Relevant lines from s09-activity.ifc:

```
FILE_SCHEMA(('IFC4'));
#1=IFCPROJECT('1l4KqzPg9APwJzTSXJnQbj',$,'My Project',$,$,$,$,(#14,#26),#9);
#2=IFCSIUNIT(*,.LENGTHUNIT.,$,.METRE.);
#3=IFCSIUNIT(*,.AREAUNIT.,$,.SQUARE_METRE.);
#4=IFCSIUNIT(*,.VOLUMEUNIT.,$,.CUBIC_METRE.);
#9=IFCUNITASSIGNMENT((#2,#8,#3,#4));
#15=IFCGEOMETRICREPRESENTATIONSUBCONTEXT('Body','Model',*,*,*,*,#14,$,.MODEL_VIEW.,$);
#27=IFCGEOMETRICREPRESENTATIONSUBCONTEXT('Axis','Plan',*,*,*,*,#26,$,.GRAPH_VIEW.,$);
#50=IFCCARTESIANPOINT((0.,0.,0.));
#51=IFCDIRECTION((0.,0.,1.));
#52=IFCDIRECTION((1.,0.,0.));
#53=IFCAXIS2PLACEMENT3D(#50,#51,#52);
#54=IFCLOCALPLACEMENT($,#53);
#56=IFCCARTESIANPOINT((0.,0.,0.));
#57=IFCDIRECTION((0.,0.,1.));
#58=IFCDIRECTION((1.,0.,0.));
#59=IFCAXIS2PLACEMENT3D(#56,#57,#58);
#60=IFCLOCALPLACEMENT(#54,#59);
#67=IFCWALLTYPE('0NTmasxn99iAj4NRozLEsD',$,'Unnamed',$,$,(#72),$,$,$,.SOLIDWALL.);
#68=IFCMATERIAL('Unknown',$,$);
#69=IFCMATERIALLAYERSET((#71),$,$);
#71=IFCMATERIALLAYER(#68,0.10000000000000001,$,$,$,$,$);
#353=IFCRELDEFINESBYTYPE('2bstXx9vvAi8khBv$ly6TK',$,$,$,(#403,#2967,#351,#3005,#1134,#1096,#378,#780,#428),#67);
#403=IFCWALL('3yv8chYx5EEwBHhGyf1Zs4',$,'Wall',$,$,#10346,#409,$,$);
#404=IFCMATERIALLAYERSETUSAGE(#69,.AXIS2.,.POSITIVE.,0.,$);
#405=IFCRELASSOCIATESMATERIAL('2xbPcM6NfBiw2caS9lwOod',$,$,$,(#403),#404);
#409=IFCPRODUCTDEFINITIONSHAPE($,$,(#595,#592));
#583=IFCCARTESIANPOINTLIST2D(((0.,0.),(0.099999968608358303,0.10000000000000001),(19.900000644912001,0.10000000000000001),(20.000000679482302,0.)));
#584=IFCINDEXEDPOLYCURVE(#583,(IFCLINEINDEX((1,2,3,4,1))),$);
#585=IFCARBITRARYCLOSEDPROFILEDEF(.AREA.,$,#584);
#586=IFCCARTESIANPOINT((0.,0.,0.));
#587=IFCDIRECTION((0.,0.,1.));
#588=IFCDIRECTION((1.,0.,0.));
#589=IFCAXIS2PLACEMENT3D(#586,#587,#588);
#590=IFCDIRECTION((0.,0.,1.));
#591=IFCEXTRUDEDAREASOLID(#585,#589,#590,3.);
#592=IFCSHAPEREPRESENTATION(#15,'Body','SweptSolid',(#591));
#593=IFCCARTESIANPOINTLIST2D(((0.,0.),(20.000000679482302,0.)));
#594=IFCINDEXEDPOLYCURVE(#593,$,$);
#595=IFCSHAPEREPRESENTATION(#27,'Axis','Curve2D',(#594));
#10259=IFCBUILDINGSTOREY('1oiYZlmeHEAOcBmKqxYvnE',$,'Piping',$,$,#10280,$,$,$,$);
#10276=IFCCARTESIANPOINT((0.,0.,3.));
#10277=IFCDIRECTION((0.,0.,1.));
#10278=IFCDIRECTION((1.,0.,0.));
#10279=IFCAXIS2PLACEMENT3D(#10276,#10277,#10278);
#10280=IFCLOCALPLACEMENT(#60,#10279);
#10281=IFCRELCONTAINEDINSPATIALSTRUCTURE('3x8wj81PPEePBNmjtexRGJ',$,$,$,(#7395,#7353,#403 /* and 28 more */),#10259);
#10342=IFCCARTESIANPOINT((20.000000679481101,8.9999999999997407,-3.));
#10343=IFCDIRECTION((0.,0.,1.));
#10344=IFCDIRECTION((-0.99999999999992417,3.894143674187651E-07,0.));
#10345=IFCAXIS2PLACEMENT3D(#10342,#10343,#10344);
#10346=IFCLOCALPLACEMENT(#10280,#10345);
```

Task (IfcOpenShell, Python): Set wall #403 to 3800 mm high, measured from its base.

```python
import ifcopenshell
import ifcopenshell.geom
import ifcopenshell.util.representation
import ifcopenshell.util.shape
import ifcopenshell.util.unit

model = ifcopenshell.open("s09-activity.ifc")
unit_scale = ifcopenshell.util.unit.calculate_unit_scale(model)
settings = ifcopenshell.geom.settings()


def volume(element):
    """Net volume in cubic metres, openings subtracted."""
    shape = ifcopenshell.geom.create_shape(settings, element)
    return ifcopenshell.util.shape.get_volume(shape.geometry)


wall = model.by_guid("3yv8chYx5EEwBHhGyf1Zs4")
before = volume(wall)

body = ifcopenshell.util.representation.get_representation(wall, "Model", "Body")
solid = body.Items[0]
old_height = solid.Depth
solid.Depth = 3.8 / unit_scale
after = volume(wall)

print(f"height {old_height:g} -> {solid.Depth:g}, volume {before:.3f} -> {after:.3f} m3")

model.write("s09-activity_rev.ifc")
```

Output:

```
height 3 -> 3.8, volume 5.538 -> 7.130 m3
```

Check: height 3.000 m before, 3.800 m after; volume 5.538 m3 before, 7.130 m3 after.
